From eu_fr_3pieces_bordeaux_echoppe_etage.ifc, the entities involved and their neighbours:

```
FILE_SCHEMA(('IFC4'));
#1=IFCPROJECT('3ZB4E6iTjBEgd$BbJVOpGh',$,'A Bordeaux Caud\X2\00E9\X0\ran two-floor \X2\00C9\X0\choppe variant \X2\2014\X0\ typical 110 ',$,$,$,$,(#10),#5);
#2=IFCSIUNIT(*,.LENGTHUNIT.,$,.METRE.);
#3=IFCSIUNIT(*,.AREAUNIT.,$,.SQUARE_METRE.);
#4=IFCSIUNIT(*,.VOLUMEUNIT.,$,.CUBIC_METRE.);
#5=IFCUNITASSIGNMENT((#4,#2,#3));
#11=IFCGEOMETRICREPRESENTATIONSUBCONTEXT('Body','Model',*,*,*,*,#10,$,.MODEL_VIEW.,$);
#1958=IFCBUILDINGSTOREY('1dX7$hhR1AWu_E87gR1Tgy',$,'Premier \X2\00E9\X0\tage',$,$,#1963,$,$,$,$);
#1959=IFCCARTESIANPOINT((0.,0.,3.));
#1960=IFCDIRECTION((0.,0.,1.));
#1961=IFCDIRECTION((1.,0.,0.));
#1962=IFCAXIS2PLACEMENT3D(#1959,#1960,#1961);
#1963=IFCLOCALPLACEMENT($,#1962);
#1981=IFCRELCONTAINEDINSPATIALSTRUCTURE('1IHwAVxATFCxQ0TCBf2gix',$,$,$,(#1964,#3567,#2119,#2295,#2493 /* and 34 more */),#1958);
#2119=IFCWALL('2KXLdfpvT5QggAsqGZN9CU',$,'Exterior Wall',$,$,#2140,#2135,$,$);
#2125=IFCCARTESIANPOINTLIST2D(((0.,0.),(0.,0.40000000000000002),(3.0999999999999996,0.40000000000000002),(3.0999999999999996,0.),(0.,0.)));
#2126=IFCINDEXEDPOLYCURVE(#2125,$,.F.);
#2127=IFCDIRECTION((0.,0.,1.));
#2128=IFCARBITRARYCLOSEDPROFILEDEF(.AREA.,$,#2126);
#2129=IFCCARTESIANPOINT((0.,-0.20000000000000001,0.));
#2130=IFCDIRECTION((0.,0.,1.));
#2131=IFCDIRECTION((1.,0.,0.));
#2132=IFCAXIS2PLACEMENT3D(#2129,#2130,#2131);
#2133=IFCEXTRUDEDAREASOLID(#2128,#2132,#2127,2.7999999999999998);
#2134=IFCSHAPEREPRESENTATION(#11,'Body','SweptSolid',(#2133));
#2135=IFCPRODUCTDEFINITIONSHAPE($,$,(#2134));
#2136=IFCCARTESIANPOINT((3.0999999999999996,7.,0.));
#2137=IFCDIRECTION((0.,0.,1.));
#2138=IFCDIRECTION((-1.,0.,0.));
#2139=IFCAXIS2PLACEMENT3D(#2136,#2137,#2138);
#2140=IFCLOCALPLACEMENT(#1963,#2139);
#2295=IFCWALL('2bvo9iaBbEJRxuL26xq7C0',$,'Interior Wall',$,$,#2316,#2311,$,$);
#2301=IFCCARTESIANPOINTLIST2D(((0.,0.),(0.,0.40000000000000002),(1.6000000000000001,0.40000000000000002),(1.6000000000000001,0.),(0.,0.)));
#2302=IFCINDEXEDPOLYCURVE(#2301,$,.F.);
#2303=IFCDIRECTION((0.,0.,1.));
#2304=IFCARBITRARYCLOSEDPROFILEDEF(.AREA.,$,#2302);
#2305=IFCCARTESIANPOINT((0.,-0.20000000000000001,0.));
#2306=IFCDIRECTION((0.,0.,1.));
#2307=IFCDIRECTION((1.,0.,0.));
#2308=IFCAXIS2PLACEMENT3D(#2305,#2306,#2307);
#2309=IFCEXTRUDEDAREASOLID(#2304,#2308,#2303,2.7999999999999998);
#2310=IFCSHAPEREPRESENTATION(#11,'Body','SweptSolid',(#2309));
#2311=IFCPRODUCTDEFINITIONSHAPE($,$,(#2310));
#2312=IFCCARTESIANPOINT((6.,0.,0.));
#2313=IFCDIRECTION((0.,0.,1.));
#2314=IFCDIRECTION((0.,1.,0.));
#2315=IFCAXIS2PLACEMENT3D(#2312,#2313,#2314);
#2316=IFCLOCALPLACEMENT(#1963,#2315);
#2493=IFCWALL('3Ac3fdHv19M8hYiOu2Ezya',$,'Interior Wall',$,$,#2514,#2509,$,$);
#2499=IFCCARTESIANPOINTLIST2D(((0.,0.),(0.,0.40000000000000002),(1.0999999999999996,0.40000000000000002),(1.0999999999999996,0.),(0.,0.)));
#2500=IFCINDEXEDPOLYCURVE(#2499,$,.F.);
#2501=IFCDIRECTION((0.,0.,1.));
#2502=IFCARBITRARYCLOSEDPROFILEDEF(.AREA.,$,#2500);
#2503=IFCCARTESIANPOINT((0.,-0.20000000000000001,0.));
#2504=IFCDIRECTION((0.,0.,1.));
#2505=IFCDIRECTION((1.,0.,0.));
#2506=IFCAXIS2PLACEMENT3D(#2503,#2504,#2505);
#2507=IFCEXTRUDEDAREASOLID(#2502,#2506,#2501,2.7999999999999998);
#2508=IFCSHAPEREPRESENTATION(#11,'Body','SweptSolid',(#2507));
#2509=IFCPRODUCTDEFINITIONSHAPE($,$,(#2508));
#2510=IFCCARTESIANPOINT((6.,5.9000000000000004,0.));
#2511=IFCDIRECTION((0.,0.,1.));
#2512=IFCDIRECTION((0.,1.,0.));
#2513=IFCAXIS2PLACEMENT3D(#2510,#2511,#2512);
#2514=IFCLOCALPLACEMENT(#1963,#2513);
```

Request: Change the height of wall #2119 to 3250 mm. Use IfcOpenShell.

```python
import ifcopenshell
import ifcopenshell.geom
import ifcopenshell.util.representation
import ifcopenshell.util.shape
import ifcopenshell.util.unit

model = ifcopenshell.open("eu_fr_3pieces_bordeaux_echoppe_etage.ifc")
unit_scale = ifcopenshell.util.unit.calculate_unit_scale(model)
settings = ifcopenshell.geom.settings()


def volume(element):
    """Net volume in cubic metres, openings subtracted."""
    shape = ifcopenshell.geom.create_shape(settings, element)
    return ifcopenshell.util.shape.get_volume(shape.geometry)


wall = model.by_guid("2KXLdfpvT5QggAsqGZN9CU")
before = volume(wall)

body = ifcopenshell.util.representation.get_representation(wall, "Model", "Body")
solid = body.Items[0]
old_height = solid.Depth
solid.Depth = 3.25 / unit_scale
after = volume(wall)

print(f"height {old_height:g} -> {solid.Depth:g}, volume {before:.3f} -> {after:.3f} m3")

model.write("eu_fr_3pieces_bordeaux_echoppe_etage_updated.ifc")
```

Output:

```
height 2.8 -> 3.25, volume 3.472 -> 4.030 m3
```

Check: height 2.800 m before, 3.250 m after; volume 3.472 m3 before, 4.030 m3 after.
